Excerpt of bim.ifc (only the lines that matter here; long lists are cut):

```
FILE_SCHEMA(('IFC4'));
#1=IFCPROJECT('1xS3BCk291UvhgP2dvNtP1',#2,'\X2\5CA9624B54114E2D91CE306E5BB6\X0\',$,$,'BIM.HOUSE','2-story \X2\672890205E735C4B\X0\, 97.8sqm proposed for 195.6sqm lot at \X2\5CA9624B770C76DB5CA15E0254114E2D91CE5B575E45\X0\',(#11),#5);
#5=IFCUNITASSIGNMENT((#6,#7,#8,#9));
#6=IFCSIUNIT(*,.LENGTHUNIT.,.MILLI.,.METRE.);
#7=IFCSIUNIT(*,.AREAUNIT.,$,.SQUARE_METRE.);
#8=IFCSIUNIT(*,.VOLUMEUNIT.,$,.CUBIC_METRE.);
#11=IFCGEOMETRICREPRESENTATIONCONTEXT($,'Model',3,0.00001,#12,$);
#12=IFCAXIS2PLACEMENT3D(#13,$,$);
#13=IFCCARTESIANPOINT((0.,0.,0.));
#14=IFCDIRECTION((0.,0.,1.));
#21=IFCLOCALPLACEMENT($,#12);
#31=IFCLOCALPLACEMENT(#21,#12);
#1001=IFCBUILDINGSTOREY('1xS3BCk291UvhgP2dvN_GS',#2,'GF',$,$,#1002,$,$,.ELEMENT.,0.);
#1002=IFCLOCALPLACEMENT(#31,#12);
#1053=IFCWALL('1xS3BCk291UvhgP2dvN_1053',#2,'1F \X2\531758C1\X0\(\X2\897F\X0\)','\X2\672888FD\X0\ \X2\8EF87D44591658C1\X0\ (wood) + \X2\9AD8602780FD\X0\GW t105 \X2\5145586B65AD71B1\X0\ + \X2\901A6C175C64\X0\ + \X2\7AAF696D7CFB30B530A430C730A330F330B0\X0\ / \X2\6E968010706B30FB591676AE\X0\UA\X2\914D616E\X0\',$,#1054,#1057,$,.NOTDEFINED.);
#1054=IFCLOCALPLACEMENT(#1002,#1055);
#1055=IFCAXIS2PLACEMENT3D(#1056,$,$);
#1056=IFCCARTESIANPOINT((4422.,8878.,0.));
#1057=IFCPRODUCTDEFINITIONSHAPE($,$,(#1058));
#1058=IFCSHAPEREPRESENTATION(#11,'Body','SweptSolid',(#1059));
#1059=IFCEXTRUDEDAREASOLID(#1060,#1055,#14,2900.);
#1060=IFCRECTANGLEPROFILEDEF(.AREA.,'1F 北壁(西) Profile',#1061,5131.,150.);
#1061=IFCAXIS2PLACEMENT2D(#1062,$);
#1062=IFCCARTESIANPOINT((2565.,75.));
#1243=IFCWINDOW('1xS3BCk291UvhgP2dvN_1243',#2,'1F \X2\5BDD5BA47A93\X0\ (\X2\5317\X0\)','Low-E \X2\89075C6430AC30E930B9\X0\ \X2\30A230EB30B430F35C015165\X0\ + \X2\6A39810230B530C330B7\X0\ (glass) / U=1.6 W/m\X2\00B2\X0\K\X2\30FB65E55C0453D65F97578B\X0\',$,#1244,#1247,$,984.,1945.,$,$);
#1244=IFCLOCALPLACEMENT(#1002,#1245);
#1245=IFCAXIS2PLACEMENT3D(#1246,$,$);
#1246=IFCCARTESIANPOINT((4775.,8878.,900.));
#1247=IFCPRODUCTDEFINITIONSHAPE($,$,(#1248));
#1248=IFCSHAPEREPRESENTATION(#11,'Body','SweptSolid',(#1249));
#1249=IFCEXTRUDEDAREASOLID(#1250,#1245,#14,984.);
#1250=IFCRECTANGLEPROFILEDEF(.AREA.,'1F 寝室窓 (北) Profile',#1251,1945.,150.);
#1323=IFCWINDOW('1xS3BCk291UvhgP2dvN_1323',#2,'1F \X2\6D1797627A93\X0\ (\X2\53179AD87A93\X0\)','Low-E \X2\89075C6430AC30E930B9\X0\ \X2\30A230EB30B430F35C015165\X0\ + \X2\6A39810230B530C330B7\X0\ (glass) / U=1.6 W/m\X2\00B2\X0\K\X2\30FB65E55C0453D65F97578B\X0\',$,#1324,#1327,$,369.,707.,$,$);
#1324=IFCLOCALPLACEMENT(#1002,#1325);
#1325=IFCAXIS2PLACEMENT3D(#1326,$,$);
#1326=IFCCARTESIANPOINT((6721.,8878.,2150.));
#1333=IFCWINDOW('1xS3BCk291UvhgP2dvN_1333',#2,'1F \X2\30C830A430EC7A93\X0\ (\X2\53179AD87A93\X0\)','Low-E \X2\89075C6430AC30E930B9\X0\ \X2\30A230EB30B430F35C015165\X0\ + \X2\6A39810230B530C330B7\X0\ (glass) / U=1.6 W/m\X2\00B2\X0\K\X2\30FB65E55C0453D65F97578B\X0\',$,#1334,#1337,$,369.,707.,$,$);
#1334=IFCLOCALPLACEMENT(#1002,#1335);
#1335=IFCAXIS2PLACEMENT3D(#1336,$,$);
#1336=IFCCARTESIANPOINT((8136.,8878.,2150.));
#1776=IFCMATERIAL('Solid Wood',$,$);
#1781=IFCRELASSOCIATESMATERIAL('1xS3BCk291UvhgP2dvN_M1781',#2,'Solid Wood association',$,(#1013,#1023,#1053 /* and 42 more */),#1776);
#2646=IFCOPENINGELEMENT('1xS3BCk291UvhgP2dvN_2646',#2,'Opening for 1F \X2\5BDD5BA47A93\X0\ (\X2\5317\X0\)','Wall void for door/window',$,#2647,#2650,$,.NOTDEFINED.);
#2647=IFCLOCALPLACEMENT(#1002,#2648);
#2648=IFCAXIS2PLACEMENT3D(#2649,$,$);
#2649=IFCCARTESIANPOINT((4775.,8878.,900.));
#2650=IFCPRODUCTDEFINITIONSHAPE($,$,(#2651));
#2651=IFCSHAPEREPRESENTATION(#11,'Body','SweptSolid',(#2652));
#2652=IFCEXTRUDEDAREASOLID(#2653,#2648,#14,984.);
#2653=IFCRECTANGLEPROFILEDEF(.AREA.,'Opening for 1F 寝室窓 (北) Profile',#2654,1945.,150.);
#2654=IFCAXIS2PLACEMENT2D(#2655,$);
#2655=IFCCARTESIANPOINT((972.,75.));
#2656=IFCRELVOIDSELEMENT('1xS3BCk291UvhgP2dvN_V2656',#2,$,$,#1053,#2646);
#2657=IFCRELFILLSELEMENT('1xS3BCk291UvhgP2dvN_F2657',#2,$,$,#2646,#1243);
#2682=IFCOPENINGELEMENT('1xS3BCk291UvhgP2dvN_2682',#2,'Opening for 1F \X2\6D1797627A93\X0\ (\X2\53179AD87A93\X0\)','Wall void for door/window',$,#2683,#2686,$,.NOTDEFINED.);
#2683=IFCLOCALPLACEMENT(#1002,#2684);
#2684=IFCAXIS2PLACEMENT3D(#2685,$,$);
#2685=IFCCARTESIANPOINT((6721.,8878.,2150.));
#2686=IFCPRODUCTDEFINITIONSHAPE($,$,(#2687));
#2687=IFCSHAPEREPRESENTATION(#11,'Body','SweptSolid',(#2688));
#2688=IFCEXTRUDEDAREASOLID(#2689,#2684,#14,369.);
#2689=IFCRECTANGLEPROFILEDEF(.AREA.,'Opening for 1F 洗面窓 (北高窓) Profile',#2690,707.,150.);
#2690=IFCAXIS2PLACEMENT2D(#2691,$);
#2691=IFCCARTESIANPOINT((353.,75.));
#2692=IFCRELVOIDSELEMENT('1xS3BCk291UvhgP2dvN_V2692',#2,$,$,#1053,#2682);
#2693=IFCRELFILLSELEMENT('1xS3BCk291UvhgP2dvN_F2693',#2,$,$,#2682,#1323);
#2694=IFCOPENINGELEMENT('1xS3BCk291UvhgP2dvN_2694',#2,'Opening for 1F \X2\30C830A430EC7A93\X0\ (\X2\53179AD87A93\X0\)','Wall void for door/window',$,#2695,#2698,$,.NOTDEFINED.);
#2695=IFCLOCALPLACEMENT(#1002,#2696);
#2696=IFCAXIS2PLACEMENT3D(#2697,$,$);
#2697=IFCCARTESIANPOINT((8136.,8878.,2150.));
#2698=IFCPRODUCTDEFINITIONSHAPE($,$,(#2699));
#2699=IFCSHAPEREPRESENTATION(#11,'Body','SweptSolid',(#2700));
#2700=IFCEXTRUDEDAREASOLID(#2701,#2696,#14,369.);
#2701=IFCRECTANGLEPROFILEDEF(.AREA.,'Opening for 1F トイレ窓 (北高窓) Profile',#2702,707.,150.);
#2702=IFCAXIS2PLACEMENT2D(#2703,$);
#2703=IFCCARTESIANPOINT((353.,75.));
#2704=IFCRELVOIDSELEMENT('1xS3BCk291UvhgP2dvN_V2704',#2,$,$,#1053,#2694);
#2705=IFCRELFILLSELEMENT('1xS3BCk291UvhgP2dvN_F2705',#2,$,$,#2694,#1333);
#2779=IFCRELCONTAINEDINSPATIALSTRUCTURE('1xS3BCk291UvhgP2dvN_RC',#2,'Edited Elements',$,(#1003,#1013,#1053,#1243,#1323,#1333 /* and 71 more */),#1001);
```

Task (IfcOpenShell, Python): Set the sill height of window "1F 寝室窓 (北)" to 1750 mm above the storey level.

```python
import numpy as np
import ifcopenshell
import ifcopenshell.api.geometry
import ifcopenshell.geom
import ifcopenshell.util.element
import ifcopenshell.util.placement
import ifcopenshell.util.shape
import ifcopenshell.util.unit

model = ifcopenshell.open("bim.ifc")
unit_scale = ifcopenshell.util.unit.calculate_unit_scale(model)

window = model.by_guid("1xS3BCk291UvhgP2dvN_1243")
opening = window.FillsVoids[0].RelatingOpeningElement
storey = ifcopenshell.util.element.get_container(window, ifc_class="IfcBuildingStorey")
level = ifcopenshell.util.placement.get_local_placement(storey.ObjectPlacement)[2, 3]

# The opening's origin need not be at the sill, so measure its lowest point.
shape = ifcopenshell.geom.create_shape(ifcopenshell.geom.settings(), opening)
bottom = ifcopenshell.util.shape.get_shape_bottom_elevation(shape, shape.geometry) / unit_scale
dz = level + 1.75 / unit_scale - bottom

shift = np.array([0.0, 0.0, dz])
# The window is not placed relative to its opening, so move both.
for product in (opening, window):
    matrix = ifcopenshell.util.placement.get_local_placement(product.ObjectPlacement)
    matrix[:3, 3] += shift
    ifcopenshell.api.geometry.edit_object_placement(model, product=product, matrix=matrix, is_si=False)

print(f"moved by {dz * unit_scale:+.3f} m")

model.write("bim_updated.ifc")
```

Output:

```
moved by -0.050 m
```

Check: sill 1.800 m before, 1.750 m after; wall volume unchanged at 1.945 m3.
